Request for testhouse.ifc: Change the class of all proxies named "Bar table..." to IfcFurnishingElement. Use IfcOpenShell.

First a look at what the model holds.

```python
import re

import ifcopenshell

model = ifcopenshell.open("testhouse.ifc")
print(model.schema)
seen = {}
for e in model.by_type("IfcBuildingElementProxy"):
    name = re.sub(r":\d+(:\d+)?$", "", e.Name or "")  # drop the element id that some exporters append
    seen[name] = seen.get(name, 0) + 1
for name, count in sorted(seen.items()):
    print(count, "x", name)
```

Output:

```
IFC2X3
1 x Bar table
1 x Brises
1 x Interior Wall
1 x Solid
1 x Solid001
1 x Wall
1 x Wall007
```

```python
import ifcopenshell
import ifcopenshell.api.root

model = ifcopenshell.open("testhouse.ifc")

proxies = [e.id() for e in model.by_type("IfcBuildingElementProxy") if (e.Name or "").startswith("Bar table")]
for step_id in proxies:
    proxy = model.by_id(step_id)
    ifcopenshell.api.root.reassign_class(model, product=proxy, ifc_class="IfcFurnishingElement")

print(sum(model.by_id(i).is_a("IfcFurnishingElement") for i in proxies), "reclassified")

model.write("testhouse_updated.ifc")
```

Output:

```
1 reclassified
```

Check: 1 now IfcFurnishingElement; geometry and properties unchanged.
